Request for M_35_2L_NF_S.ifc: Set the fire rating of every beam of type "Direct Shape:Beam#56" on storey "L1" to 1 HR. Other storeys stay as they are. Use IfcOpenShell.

First a look at what the model holds.

```python
import ifcopenshell
import ifcopenshell.util.element

model = ifcopenshell.open("M_35_2L_NF_S.ifc")
print(model.schema)
storey = next(s for s in model.by_type("IfcBuildingStorey") if s.Name == "L1")
beams = [e for e in ifcopenshell.util.element.get_decomposition(storey) if e.is_a("IfcBeam")]
seen = {}
for e in beams:
    element_type = ifcopenshell.util.element.get_type(e)
    key = (element_type.Name if element_type != e and element_type else None, ifcopenshell.util.element.get_pset(e, "Pset_BeamCommon", "FireRating"))
    seen[key] = seen.get(key, 0) + 1
for (name, value), count in sorted(seen.items(), key=str):
    print(count, "x", name, "|", value)
```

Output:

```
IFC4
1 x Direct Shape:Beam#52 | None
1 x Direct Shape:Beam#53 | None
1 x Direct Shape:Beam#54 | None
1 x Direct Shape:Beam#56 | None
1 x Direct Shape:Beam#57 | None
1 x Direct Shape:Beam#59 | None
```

```python
import ifcopenshell
import ifcopenshell.api.pset
import ifcopenshell.util.element

model = ifcopenshell.open("M_35_2L_NF_S.ifc")

storey = next(s for s in model.by_type("IfcBuildingStorey") if s.Name == "L1")
beams = [e for e in ifcopenshell.util.element.get_decomposition(storey) if e.is_a("IfcBeam")]

count = 0
for e in beams:
    element_type = ifcopenshell.util.element.get_type(e)
    if element_type in (None, e) or element_type.Name != "Direct Shape:Beam#56":
        continue
    # add_pset returns the element's existing set when there is one.
    pset = ifcopenshell.api.pset.add_pset(model, product=e, name="Pset_BeamCommon")
    ifcopenshell.api.pset.edit_pset(model, pset=pset, properties={"FireRating": "1 HR"})
    count += 1

print(count, "beams updated")

model.write("M_35_2L_NF_S_v2.ifc")
```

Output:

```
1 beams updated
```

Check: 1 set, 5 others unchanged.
